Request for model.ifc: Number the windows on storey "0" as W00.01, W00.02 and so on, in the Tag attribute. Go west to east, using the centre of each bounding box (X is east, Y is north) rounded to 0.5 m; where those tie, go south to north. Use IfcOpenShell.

First a look at what the model holds.

```python
import ifcopenshell
import ifcopenshell.util.element
import ifcopenshell.util.placement

model = ifcopenshell.open("model.ifc")
print(model.schema)
storey = next(s for s in model.by_type("IfcBuildingStorey") if s.Name == "0")
windows = [e for e in ifcopenshell.util.element.get_decomposition(storey) if e.is_a("IfcWindow")]
for e in sorted(windows, key=lambda e: e.id()):
    origin = ifcopenshell.util.placement.get_local_placement(e.ObjectPlacement)[:3, 3]
    print(e.id(), e.Tag, e.Name, origin.round(2) + 0.0, sep=" | ")
```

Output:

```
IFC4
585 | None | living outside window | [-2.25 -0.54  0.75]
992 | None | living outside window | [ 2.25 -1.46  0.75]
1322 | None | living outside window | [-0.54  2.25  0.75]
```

```python
import ifcopenshell
import ifcopenshell.geom
import ifcopenshell.util.element
import ifcopenshell.util.shape

model = ifcopenshell.open("model.ifc")
settings = ifcopenshell.geom.settings()
settings.set("use-world-coords", True)


def centre(element):
    shape = ifcopenshell.geom.create_shape(settings, element)
    return ifcopenshell.util.shape.get_bbox_centroid(shape.geometry)


storey = next(s for s in model.by_type("IfcBuildingStorey") if s.Name == "0")
windows = [e for e in ifcopenshell.util.element.get_decomposition(storey) if e.is_a("IfcWindow")]

# Insertion points can sit at a corner or the storey origin, so sort by the geometry (in metres).
centres = {e: centre(e) for e in windows}
windows.sort(key=lambda e: (round(centres[e][0] / 0.5), centres[e][1]))

for i, e in enumerate(windows, start=1):
    number = f"W00.{i:02d}"
    e.Tag = number
    print(e.id(), number)

model.write("model_rev.ifc")
```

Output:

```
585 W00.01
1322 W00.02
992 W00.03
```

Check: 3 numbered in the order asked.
